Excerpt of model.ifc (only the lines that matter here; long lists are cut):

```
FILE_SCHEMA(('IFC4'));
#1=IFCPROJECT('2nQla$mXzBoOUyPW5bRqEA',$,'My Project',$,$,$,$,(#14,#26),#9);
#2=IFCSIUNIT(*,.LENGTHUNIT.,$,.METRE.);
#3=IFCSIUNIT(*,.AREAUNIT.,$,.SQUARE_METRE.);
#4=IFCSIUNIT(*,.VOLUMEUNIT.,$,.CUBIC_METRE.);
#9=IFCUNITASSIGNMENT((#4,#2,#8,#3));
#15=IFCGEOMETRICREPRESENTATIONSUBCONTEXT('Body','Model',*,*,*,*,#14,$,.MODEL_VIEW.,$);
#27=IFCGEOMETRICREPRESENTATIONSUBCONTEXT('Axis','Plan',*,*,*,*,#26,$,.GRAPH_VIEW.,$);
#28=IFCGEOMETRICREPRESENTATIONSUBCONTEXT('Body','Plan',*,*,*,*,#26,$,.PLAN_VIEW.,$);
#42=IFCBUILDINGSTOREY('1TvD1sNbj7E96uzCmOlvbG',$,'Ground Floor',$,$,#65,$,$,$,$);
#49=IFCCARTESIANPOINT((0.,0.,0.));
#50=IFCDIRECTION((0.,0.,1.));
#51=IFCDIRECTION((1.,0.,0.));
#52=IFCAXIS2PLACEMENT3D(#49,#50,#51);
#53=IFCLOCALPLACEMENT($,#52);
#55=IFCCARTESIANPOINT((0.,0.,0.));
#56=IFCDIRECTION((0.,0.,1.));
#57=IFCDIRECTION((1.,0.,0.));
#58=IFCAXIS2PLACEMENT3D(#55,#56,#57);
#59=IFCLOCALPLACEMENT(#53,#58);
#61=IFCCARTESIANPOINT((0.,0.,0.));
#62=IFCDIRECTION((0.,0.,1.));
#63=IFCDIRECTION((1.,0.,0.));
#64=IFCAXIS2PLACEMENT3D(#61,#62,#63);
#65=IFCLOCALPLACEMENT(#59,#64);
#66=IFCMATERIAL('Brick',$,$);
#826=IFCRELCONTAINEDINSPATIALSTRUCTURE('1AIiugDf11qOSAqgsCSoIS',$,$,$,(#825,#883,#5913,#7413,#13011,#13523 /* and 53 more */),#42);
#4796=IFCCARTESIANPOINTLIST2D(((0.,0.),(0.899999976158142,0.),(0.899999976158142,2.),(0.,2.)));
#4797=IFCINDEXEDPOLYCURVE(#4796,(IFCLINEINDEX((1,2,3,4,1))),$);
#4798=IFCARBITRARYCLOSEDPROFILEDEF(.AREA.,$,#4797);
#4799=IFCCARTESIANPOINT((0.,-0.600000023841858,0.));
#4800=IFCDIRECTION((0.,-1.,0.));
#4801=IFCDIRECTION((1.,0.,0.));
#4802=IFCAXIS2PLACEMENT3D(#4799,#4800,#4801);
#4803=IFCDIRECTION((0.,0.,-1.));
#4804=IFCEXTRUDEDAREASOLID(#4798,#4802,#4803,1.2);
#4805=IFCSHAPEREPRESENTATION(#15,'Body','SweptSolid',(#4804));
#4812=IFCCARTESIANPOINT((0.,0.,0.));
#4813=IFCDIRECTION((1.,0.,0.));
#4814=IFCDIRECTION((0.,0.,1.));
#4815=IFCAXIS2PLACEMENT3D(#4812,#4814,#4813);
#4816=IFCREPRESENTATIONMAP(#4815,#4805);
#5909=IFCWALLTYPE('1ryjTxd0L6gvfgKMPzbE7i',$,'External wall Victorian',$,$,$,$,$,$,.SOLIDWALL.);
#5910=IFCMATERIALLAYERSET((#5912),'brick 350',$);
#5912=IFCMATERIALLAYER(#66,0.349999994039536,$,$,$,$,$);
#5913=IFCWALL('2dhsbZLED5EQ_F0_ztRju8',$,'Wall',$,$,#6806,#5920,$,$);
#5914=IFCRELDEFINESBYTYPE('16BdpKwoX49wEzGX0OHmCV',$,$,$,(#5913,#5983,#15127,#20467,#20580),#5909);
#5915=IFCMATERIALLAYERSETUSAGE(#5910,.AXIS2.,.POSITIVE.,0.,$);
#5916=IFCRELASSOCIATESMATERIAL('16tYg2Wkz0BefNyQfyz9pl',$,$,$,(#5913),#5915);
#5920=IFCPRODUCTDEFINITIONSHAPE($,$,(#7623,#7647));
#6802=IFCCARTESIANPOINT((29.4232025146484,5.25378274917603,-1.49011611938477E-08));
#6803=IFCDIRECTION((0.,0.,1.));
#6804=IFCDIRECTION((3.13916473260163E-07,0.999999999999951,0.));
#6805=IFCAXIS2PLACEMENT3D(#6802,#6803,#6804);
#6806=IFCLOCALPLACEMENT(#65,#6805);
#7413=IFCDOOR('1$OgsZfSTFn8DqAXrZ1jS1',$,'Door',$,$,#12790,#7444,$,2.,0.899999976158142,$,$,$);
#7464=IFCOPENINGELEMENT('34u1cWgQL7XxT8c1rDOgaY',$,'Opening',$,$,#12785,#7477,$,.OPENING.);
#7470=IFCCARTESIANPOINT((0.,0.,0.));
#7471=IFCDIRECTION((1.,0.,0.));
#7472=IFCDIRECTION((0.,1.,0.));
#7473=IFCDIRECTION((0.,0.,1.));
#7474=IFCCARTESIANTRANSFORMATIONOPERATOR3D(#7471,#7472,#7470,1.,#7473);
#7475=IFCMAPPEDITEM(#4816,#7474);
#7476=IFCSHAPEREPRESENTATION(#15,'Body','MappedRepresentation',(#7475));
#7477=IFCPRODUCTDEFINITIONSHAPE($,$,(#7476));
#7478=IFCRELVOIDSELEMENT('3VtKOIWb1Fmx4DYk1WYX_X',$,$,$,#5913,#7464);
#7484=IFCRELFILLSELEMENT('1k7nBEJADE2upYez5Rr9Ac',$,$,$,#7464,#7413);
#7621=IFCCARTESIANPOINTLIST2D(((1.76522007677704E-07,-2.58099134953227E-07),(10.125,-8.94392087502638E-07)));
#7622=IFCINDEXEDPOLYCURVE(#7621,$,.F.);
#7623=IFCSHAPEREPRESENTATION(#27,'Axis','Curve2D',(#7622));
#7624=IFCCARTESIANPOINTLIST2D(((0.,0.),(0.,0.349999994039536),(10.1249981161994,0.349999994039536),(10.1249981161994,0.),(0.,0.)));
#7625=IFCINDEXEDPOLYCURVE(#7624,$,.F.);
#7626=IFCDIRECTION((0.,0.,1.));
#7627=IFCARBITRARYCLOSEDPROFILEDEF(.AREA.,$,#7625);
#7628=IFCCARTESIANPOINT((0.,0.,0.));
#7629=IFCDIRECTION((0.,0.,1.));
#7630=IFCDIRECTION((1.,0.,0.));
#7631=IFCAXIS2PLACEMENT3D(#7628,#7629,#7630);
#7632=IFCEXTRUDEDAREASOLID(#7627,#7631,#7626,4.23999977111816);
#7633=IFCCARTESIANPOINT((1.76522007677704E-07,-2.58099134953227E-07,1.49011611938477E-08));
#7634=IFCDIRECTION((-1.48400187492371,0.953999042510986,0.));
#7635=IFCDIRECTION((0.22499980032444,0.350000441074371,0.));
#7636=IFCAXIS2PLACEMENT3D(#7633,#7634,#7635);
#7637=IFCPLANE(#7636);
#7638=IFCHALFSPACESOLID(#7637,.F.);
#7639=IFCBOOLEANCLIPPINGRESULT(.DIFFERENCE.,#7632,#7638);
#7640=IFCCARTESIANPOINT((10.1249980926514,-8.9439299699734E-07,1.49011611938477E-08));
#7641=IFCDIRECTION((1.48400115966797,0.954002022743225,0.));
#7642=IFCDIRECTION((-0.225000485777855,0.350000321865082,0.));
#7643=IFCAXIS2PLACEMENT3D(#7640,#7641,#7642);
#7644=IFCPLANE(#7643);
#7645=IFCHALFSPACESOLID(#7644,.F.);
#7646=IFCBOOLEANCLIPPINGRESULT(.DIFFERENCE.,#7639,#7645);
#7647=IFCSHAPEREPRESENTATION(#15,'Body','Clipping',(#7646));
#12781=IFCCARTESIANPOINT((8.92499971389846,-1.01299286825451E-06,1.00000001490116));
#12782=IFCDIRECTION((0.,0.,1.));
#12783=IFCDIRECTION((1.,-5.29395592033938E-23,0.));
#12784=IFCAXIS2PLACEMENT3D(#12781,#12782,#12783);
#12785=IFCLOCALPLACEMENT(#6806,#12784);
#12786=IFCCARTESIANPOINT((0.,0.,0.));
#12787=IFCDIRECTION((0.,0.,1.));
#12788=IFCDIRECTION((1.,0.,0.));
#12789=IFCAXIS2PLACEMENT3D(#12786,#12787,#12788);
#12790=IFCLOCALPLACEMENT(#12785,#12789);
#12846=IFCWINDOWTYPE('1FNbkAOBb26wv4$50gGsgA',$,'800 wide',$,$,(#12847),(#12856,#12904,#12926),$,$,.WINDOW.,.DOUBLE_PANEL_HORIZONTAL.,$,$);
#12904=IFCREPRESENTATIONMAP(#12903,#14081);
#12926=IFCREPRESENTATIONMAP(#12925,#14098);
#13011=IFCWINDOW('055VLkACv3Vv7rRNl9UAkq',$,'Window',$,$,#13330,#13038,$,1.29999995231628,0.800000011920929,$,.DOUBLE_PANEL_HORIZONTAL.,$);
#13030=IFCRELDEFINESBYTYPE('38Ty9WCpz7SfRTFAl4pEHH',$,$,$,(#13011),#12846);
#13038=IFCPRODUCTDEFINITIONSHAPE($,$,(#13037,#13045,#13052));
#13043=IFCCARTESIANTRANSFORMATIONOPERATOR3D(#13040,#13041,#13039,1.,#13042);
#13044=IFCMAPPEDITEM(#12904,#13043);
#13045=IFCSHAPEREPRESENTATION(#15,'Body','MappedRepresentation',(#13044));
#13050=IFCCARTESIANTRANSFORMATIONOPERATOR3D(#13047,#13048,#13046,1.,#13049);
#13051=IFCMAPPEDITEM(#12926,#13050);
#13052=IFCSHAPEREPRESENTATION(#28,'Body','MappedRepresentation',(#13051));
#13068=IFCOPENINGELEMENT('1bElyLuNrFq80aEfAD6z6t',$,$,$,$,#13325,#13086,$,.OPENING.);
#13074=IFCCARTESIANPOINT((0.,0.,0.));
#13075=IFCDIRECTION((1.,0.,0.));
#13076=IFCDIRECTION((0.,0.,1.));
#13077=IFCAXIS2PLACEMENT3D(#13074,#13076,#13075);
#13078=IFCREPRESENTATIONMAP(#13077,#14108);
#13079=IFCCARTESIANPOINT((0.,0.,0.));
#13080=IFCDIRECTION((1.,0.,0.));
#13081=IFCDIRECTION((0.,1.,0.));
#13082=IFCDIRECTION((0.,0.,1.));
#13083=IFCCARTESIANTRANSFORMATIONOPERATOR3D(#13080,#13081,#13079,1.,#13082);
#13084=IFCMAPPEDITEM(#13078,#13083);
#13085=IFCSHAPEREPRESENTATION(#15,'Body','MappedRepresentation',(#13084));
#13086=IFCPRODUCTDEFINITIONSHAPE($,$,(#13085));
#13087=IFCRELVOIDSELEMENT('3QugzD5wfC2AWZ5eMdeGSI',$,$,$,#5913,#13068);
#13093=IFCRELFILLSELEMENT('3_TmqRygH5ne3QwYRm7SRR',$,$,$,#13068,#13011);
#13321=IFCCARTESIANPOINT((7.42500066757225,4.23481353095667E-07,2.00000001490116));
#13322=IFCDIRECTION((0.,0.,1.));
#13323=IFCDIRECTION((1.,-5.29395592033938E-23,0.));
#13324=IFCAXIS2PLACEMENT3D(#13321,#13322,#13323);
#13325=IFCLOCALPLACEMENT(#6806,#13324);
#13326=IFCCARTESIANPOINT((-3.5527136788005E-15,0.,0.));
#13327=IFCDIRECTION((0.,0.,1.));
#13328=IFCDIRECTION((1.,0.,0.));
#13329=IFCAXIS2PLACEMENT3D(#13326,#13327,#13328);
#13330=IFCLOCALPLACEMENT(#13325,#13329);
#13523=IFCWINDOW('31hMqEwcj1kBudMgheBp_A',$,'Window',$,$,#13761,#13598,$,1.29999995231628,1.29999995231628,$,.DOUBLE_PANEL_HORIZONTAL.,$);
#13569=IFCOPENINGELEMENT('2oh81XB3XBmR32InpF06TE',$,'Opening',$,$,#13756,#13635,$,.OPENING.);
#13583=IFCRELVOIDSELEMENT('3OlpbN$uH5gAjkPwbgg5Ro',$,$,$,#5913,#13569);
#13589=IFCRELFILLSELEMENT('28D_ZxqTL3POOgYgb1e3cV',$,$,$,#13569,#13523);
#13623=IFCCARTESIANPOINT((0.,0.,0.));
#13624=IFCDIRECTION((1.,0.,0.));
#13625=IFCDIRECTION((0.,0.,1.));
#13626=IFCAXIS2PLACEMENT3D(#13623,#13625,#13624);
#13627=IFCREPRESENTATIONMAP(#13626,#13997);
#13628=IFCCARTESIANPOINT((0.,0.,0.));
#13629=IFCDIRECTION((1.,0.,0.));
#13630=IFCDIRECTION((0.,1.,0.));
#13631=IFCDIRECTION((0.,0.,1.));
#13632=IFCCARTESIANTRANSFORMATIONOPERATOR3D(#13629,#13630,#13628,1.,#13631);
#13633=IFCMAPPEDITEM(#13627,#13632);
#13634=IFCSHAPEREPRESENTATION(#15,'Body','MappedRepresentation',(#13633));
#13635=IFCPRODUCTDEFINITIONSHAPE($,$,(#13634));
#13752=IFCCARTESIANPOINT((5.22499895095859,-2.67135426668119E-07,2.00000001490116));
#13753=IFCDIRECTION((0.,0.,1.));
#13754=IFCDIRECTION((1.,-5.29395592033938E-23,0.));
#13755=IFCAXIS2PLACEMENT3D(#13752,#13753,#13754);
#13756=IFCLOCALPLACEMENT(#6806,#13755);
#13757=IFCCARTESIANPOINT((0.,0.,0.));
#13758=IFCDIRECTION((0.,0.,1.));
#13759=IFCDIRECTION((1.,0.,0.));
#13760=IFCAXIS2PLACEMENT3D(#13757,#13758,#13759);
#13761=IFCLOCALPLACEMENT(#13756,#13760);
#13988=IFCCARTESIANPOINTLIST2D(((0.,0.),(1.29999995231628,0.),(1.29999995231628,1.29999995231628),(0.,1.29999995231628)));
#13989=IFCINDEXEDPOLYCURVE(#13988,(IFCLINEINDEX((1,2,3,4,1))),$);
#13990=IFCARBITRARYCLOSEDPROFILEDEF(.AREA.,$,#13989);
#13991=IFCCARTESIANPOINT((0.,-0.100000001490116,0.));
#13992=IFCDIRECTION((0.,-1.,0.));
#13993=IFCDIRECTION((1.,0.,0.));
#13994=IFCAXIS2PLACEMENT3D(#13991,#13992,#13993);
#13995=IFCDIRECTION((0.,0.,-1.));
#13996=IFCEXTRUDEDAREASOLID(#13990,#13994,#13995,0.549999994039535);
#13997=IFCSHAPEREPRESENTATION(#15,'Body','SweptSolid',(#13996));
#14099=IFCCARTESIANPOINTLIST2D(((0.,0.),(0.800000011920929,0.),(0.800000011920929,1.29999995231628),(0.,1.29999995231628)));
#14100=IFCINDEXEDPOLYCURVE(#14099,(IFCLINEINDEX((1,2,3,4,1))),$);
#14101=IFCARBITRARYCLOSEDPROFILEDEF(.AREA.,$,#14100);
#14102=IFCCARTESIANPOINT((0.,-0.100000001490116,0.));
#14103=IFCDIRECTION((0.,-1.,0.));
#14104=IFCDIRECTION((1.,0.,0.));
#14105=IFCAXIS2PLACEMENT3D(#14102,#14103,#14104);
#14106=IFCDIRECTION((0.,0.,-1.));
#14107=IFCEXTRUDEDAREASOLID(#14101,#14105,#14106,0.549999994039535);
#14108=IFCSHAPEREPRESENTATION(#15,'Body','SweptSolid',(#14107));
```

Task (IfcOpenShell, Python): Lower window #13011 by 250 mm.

```python
import numpy as np
import ifcopenshell
import ifcopenshell.api.geometry
import ifcopenshell.util.placement
import ifcopenshell.util.unit

model = ifcopenshell.open("model.ifc")
unit_scale = ifcopenshell.util.unit.calculate_unit_scale(model)

window = model.by_guid("055VLkACv3Vv7rRNl9UAkq")
opening = window.FillsVoids[0].RelatingOpeningElement
dz = -0.25 / unit_scale

shift = np.array([0.0, 0.0, dz])
# The window is placed relative to its opening, so it follows when the opening moves.
matrix = ifcopenshell.util.placement.get_local_placement(opening.ObjectPlacement)
matrix[:3, 3] += shift
ifcopenshell.api.geometry.edit_object_placement(
    model, product=opening, matrix=matrix, is_si=False, should_transform_children=True
)

print(f"moved by {dz * unit_scale:+.3f} m")

model.write("model_edited.ifc")
```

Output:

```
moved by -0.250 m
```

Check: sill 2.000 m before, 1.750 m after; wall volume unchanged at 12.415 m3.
